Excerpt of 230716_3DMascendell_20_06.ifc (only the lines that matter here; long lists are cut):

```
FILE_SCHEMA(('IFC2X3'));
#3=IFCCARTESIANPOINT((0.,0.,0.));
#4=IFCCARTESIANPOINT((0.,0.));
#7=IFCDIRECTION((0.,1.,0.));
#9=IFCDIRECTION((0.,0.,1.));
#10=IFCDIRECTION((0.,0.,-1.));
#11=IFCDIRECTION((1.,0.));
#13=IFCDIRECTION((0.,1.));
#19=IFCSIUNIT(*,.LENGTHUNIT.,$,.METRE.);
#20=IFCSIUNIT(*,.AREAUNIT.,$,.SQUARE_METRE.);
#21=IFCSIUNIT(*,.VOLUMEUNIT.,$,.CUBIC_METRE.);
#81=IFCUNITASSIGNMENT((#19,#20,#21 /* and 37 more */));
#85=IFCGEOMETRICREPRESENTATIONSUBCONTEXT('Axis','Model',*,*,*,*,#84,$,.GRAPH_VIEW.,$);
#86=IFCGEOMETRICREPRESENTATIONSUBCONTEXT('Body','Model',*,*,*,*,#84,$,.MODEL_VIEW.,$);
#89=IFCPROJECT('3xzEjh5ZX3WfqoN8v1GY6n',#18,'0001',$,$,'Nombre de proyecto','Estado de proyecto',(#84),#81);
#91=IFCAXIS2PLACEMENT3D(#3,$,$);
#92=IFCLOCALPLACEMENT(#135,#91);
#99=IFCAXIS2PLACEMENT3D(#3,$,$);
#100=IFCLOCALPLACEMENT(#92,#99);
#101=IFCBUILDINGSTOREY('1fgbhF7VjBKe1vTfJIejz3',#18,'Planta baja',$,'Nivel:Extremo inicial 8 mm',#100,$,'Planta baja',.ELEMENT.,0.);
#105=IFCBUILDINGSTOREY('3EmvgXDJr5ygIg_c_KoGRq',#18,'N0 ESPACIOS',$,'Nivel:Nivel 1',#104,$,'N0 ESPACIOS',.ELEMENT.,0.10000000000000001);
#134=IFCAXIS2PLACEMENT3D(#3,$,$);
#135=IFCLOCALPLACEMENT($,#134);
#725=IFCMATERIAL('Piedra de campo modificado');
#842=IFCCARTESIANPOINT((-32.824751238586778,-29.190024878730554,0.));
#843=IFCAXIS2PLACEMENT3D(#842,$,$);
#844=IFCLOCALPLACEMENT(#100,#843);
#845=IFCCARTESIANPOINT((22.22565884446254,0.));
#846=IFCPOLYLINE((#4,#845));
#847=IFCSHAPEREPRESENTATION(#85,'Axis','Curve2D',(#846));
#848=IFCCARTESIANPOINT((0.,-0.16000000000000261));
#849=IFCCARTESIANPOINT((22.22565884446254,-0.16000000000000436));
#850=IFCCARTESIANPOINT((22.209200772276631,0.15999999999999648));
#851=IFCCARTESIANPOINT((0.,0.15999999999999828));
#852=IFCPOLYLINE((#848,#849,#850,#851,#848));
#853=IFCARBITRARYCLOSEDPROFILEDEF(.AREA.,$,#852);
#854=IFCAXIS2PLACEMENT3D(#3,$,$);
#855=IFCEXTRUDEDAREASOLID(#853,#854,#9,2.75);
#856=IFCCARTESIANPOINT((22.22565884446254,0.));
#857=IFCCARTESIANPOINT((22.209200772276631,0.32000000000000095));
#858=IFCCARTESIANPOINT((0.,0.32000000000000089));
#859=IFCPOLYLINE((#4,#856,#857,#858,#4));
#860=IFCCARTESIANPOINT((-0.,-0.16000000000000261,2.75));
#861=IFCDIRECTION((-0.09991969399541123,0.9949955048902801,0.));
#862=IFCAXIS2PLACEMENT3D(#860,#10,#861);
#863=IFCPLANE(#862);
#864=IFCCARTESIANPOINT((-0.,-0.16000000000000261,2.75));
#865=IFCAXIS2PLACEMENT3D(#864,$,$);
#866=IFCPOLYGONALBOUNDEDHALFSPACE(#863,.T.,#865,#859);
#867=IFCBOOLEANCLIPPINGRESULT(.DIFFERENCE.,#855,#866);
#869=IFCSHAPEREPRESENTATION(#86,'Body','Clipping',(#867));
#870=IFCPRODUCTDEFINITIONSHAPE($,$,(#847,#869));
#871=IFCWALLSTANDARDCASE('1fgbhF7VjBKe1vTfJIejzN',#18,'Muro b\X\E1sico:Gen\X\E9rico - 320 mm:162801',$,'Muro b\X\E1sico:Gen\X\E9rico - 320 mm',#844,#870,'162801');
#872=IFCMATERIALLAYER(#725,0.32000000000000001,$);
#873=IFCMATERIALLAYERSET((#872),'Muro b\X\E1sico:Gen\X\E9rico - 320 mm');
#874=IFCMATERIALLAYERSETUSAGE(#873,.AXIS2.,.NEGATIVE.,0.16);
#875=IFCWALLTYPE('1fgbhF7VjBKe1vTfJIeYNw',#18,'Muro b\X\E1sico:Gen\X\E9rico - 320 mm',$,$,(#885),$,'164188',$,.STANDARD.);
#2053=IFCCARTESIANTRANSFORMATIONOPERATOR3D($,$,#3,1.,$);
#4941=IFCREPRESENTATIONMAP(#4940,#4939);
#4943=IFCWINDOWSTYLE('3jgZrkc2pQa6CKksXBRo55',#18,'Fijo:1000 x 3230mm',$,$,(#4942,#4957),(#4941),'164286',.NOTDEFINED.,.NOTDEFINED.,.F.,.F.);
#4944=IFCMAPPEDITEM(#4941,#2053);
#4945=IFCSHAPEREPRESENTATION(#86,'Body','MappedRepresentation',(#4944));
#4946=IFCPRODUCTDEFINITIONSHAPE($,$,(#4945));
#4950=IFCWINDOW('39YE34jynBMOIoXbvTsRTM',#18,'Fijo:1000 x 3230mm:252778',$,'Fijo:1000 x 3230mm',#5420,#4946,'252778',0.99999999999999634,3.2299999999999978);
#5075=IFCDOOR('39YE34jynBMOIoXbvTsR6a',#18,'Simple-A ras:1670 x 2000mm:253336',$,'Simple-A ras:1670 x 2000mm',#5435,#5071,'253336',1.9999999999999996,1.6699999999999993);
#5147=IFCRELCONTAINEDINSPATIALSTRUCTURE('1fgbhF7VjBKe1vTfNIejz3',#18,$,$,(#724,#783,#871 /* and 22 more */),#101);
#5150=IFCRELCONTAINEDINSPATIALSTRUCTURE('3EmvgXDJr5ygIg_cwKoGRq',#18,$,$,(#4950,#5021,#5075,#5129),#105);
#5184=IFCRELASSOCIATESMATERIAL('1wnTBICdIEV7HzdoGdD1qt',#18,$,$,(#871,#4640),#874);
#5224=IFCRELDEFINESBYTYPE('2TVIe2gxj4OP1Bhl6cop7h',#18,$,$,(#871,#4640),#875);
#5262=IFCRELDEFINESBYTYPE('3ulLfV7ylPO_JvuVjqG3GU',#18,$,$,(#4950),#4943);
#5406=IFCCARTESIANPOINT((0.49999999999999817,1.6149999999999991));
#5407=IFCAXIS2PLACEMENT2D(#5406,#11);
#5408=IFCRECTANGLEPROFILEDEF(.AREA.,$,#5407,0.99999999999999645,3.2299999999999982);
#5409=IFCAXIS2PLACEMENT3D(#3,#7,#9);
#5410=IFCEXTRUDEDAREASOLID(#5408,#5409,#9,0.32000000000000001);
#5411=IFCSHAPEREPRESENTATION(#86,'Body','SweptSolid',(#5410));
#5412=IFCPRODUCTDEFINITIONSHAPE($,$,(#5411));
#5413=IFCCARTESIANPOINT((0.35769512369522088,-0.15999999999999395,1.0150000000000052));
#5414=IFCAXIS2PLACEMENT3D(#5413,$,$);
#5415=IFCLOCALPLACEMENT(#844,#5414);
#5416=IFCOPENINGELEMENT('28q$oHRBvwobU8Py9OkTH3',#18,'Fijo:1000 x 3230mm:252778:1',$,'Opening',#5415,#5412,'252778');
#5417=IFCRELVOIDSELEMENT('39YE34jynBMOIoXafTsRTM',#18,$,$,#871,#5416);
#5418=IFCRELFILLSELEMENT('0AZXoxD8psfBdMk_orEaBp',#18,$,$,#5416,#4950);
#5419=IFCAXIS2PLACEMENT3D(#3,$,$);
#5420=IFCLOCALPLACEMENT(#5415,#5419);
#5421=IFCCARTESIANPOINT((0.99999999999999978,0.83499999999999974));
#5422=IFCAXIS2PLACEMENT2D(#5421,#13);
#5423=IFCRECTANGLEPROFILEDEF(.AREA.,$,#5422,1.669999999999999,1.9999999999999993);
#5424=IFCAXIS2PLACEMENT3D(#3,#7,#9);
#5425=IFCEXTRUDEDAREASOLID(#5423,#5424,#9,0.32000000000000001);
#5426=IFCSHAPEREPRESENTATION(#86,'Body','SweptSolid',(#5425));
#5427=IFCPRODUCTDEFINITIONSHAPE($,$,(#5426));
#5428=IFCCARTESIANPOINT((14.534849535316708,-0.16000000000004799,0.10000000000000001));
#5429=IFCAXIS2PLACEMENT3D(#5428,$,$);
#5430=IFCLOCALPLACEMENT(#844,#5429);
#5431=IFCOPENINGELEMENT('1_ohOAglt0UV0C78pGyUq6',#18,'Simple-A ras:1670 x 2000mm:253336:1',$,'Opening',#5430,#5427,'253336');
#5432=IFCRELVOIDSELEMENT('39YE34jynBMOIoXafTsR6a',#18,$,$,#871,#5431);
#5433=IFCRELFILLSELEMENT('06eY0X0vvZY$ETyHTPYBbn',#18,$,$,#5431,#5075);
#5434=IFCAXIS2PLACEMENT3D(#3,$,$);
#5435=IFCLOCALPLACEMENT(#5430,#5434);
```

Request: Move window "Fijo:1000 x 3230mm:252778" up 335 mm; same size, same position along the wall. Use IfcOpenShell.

```python
import numpy as np
import ifcopenshell
import ifcopenshell.api.geometry
import ifcopenshell.util.placement
import ifcopenshell.util.unit

model = ifcopenshell.open("230716_3DMascendell_20_06.ifc")
unit_scale = ifcopenshell.util.unit.calculate_unit_scale(model)

window = model.by_guid("39YE34jynBMOIoXbvTsRTM")
opening = window.FillsVoids[0].RelatingOpeningElement
dz = 0.335 / unit_scale

shift = np.array([0.0, 0.0, dz])
# The window is placed relative to its opening, so it follows when the opening moves.
matrix = ifcopenshell.util.placement.get_local_placement(opening.ObjectPlacement)
matrix[:3, 3] += shift
ifcopenshell.api.geometry.edit_object_placement(
    model, product=opening, matrix=matrix, is_si=False, should_transform_children=True
)

print(f"moved by {dz * unit_scale:+.3f} m")

model.write("230716_3DMascendell_20_06-out.ifc")
```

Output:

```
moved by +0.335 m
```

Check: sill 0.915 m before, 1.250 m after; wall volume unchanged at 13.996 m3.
